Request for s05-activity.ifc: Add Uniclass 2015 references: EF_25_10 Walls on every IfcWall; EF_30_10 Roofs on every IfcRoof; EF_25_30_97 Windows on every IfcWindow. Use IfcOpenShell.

First a look at what the model holds.

```python
import ifcopenshell

model = ifcopenshell.open("s05-activity.ifc")
print(model.schema)
print("classifications:", [c.Name for c in model.by_type("IfcClassification")])
for ifc_class in ("IfcDoor", "IfcRoof", "IfcStair", "IfcWall", "IfcWindow"):
    print(ifc_class, len(model.by_type(ifc_class)))
```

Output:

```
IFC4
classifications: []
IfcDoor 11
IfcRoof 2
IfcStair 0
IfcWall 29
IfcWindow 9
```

```python
import ifcopenshell
import ifcopenshell.api.classification

model = ifcopenshell.open("s05-activity.ifc")

system = ifcopenshell.api.classification.add_classification(model, classification="Uniclass 2015")

codes = {
    "IfcWall": ("EF_25_10", "Walls"),
    "IfcRoof": ("EF_30_10", "Roofs"),
    "IfcWindow": ("EF_25_30_97", "Windows"),
}
for ifc_class, (code, name) in codes.items():
    products = model.by_type(ifc_class)
    ifcopenshell.api.classification.add_reference(
        model, products=products, classification=system, identification=code, name=name
    )
    print(code, len(products))

model.write("s05-activity-out.ifc")
```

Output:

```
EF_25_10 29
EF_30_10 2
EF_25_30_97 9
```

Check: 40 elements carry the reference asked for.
